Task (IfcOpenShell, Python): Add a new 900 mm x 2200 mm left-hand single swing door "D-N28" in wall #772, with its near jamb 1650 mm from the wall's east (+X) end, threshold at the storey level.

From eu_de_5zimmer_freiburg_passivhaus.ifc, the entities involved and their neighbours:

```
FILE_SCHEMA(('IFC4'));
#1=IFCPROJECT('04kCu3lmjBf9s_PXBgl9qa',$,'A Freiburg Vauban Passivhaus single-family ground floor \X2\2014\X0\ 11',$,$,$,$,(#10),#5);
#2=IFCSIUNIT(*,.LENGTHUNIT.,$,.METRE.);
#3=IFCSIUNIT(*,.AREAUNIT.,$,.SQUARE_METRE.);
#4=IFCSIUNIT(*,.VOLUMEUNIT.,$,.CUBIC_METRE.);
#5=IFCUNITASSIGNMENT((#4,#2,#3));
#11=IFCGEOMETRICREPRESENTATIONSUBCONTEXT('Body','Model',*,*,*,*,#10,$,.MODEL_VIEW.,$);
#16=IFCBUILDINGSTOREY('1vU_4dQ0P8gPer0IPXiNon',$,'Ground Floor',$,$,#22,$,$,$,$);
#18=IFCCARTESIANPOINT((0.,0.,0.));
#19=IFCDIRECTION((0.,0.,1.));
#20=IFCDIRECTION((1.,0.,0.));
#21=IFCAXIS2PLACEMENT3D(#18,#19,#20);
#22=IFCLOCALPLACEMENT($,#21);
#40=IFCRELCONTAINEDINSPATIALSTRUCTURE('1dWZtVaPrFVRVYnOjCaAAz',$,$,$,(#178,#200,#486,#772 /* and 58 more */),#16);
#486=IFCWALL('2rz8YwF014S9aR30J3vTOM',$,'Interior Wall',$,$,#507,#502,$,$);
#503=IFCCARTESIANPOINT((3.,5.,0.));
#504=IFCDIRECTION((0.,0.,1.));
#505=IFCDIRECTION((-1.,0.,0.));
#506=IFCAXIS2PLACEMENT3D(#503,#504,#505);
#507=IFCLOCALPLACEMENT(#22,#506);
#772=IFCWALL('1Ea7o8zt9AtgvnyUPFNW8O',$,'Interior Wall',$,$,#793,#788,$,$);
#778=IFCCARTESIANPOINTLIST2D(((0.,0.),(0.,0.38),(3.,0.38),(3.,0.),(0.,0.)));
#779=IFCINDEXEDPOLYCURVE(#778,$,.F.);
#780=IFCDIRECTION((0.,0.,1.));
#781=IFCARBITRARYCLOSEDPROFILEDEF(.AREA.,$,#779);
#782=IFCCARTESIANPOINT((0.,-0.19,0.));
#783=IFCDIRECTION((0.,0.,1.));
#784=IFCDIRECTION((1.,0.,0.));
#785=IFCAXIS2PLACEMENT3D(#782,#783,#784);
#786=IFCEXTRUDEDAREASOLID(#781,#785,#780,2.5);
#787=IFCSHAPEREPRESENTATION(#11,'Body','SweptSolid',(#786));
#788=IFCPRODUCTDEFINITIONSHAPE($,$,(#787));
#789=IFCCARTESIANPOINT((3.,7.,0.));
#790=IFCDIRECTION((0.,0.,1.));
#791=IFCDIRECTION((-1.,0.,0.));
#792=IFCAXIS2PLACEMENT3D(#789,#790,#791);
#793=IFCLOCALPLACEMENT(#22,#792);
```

```python
import numpy as np
import ifcopenshell
import ifcopenshell.api.feature
import ifcopenshell.api.geometry
import ifcopenshell.api.root
import ifcopenshell.api.spatial
import ifcopenshell.geom
import ifcopenshell.util.element
import ifcopenshell.util.placement
import ifcopenshell.util.representation
import ifcopenshell.util.shape
import ifcopenshell.util.unit

model = ifcopenshell.open("eu_de_5zimmer_freiburg_passivhaus.ifc")
unit_scale = ifcopenshell.util.unit.calculate_unit_scale(model)
settings = ifcopenshell.geom.settings()


def volume(element):
    """Net volume in cubic metres, openings subtracted."""
    shape = ifcopenshell.geom.create_shape(settings, element)
    return ifcopenshell.util.shape.get_volume(shape.geometry)


wall = model.by_guid("1Ea7o8zt9AtgvnyUPFNW8O")
storey = ifcopenshell.util.element.get_container(wall, ifc_class="IfcBuildingStorey")
context = ifcopenshell.util.representation.get_context(model, "Model", "Body", "MODEL_VIEW")
before = volume(wall)

width, height, from_end, sill = 0.9, 2.2, 1.65, 0.0  # metres

# The wall runs along its own X axis, and the end named is its -X end.
wall_shape = ifcopenshell.geom.create_shape(settings, wall)
x, y, z = ifcopenshell.util.shape.get_vertices(wall_shape.geometry).T
start = x.min() + from_end
face, thickness = float(y.min()), float(y.max() - y.min())
wall_matrix = ifcopenshell.util.placement.get_local_placement(wall.ObjectPlacement)
level = ifcopenshell.util.placement.get_local_placement(storey.ObjectPlacement)[2, 3]


def in_wall(x, y):
    """Placement at x, y metres in the wall's axes, at sill height."""
    matrix = wall_matrix.copy()
    matrix[:, 3] = wall_matrix @ np.array([x / unit_scale, y / unit_scale, 0.0, 1.0])
    matrix[2, 3] = level + sill / unit_scale
    return matrix


# Opening: a box that overshoots both wall faces by 50 mm.
opening = ifcopenshell.api.root.create_entity(model, ifc_class="IfcOpeningElement", predefined_type="OPENING")
box = ifcopenshell.api.geometry.add_wall_representation(
    model, context=context, length=width, height=height, thickness=thickness + 0.1
)
ifcopenshell.api.geometry.assign_representation(model, product=opening, representation=box)
ifcopenshell.api.geometry.edit_object_placement(model, product=opening, matrix=in_wall(start, face - 0.05), is_si=False)
ifcopenshell.api.feature.add_feature(model, feature=opening, element=wall)

door = ifcopenshell.api.root.create_entity(model, ifc_class="IfcDoor", name="D-N28", predefined_type="DOOR")
door.OverallWidth, door.OverallHeight = width / unit_scale, height / unit_scale
door.OperationType = "SINGLE_SWING_LEFT"
body = ifcopenshell.api.geometry.add_door_representation(
    model,
    context=context,
    overall_width=door.OverallWidth,
    overall_height=door.OverallHeight,
    operation_type="SINGLE_SWING_LEFT",
    lining_properties={"LiningDepth": thickness / unit_scale, "ThresholdDepth": thickness / unit_scale},
)
ifcopenshell.api.geometry.assign_representation(model, product=door, representation=body)
ifcopenshell.api.spatial.assign_container(model, products=[door], relating_structure=storey)
ifcopenshell.api.feature.add_filling(model, opening=opening, element=door)

# The lining spans the wall, so the door starts at the wall face.
ifcopenshell.api.geometry.edit_object_placement(model, product=door, matrix=in_wall(start, face), is_si=False)

after = volume(wall)

print(f"wall volume {before:.3f} -> {after:.3f} m3")

model.write("eu_de_5zimmer_freiburg_passivhaus_updated.ifc")
```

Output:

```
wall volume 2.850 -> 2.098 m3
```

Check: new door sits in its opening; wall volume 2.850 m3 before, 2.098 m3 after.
